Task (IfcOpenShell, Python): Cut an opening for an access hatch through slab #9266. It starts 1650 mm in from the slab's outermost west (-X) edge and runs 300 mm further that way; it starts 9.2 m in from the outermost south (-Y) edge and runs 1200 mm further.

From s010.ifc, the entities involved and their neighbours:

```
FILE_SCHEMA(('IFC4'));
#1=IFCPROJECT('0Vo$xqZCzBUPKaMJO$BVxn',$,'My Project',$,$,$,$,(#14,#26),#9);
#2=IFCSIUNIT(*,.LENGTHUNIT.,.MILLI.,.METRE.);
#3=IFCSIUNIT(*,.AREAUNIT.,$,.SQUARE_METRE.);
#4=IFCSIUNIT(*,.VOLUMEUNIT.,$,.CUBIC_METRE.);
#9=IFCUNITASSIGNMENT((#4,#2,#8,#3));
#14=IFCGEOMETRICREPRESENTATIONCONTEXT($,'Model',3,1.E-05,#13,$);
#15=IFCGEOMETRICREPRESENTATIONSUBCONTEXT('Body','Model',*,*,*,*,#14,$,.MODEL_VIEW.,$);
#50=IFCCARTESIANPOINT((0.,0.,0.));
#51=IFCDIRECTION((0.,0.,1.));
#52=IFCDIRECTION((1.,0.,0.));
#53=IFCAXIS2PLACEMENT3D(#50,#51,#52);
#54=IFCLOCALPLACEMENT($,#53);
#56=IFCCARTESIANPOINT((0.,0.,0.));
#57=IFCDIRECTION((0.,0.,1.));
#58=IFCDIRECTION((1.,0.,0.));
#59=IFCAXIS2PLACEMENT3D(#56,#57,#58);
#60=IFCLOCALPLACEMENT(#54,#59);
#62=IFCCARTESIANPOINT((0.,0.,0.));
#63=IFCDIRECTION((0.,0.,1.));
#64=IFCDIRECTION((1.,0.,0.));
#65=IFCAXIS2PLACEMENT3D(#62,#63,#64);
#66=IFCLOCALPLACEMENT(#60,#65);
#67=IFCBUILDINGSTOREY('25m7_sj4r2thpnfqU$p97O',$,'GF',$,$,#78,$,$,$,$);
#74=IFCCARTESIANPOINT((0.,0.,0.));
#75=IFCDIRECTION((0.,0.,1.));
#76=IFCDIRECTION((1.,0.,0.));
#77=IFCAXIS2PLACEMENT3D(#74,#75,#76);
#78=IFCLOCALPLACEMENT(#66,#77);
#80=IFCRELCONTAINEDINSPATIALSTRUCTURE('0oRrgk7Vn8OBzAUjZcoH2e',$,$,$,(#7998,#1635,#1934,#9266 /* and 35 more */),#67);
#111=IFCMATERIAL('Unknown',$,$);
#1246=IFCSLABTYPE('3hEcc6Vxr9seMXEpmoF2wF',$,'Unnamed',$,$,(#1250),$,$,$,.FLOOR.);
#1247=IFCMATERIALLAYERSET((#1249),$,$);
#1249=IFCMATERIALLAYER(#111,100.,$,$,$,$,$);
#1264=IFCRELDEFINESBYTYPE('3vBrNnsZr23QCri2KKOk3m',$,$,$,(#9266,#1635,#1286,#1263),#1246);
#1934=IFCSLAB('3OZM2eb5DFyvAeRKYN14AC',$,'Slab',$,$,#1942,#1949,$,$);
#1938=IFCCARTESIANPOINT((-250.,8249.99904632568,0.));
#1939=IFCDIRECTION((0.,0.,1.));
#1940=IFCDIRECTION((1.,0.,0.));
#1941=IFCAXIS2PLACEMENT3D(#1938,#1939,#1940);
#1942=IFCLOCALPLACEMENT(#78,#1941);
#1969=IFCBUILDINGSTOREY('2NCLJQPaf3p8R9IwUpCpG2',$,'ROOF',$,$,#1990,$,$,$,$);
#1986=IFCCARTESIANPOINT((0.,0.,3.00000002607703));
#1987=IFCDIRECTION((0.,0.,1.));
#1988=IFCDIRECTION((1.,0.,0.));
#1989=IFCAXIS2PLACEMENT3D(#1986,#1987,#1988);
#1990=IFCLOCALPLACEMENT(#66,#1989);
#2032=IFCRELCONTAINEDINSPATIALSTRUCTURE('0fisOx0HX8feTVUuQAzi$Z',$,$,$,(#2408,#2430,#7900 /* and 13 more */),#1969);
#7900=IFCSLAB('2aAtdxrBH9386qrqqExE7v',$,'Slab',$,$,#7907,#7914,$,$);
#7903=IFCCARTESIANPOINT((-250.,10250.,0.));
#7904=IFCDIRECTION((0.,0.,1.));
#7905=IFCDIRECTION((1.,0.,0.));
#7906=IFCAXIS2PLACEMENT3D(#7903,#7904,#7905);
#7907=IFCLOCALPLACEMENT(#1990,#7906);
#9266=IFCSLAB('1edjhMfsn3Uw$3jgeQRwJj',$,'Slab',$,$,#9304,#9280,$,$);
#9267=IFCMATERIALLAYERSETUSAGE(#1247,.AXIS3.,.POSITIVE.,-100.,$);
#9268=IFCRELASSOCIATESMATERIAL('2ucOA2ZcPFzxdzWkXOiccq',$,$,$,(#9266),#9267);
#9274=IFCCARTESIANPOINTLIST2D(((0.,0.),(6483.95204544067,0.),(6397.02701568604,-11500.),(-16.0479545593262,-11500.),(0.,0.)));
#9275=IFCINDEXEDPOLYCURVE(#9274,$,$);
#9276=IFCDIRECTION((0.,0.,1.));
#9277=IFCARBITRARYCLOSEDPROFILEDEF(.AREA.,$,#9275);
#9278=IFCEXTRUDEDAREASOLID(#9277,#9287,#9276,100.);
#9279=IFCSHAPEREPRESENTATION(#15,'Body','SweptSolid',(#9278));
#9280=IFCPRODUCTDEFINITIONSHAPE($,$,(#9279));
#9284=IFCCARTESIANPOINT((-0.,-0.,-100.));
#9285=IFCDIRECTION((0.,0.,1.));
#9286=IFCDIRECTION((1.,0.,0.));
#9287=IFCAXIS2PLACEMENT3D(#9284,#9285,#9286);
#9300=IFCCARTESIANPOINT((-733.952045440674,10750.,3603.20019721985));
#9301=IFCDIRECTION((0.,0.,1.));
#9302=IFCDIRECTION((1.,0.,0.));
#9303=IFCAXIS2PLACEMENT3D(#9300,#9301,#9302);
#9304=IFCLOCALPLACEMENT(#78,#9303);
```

```python
import numpy as np
import ifcopenshell
import ifcopenshell.api.feature
import ifcopenshell.api.geometry
import ifcopenshell.api.root
import ifcopenshell.geom
import ifcopenshell.util.placement
import ifcopenshell.util.representation
import ifcopenshell.util.shape
import ifcopenshell.util.unit

model = ifcopenshell.open("s010.ifc")
unit_scale = ifcopenshell.util.unit.calculate_unit_scale(model)
settings = ifcopenshell.geom.settings()


def volume(element):
    """Net volume in cubic metres, openings subtracted."""
    shape = ifcopenshell.geom.create_shape(settings, element)
    return ifcopenshell.util.shape.get_volume(shape.geometry)


slab = model.by_id(9266)
before = volume(slab)

# Extent in the slab's own axes, in metres. The edges named are its -X and -Y sides.
slab_shape = ifcopenshell.geom.create_shape(settings, slab)
vertices = ifcopenshell.util.shape.get_vertices(slab_shape.geometry)
x_min, y_min, bottom = vertices.min(axis=0)
top = vertices[:, 2].max()

opening = ifcopenshell.api.root.create_entity(model, ifc_class="IfcOpeningElement", name="Access hatch opening", predefined_type="OPENING")
context = ifcopenshell.util.representation.get_context(model, "Model", "Body", "MODEL_VIEW")
width, depth = 0.3, 1.2
outline = [(0.0, 0.0), (width, 0.0), (width, depth), (0.0, depth), (0.0, 0.0)]
# Overshoot both faces by 50 mm so the cut is clean.
shape = ifcopenshell.api.geometry.add_slab_representation(
    model, context=context, depth=top - bottom + 0.1, polyline=outline
)
ifcopenshell.api.geometry.assign_representation(model, product=opening, representation=shape)

matrix = ifcopenshell.util.placement.get_local_placement(slab.ObjectPlacement)
matrix[:, 3] = matrix @ np.append(np.array([x_min + 1.65, y_min + 9.2, bottom - 0.05]) / unit_scale, 1.0)
ifcopenshell.api.geometry.edit_object_placement(model, product=opening, matrix=matrix, is_si=False)
ifcopenshell.api.feature.add_feature(model, feature=opening, element=slab)

after = volume(slab)

print(f"slab volume {before:.3f} -> {after:.3f} m3")

model.write("s010-out.ifc")
```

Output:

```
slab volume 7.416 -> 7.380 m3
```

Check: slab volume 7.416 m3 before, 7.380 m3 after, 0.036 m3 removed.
